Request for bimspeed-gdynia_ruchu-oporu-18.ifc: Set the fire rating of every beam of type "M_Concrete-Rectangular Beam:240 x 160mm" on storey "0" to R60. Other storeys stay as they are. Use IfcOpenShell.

First a look at what the model holds.

```python
import ifcopenshell
import ifcopenshell.util.element

model = ifcopenshell.open("bimspeed-gdynia_ruchu-oporu-18.ifc")
print(model.schema)
storey = next(s for s in model.by_type("IfcBuildingStorey") if s.Name == "0")
beams = [e for e in ifcopenshell.util.element.get_decomposition(storey) if e.is_a("IfcBeam")]
seen = {}
for e in beams:
    element_type = ifcopenshell.util.element.get_type(e)
    key = (element_type.Name if element_type != e and element_type else None, ifcopenshell.util.element.get_pset(e, "Pset_BeamCommon", "FireRating"))
    seen[key] = seen.get(key, 0) + 1
for (name, value), count in sorted(seen.items(), key=str):
    print(count, "x", name, "|", value)
```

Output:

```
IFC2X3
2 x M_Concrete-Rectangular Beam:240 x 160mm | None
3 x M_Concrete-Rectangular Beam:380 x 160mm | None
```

```python
import ifcopenshell
import ifcopenshell.api.pset
import ifcopenshell.util.element

model = ifcopenshell.open("bimspeed-gdynia_ruchu-oporu-18.ifc")

storey = next(s for s in model.by_type("IfcBuildingStorey") if s.Name == "0")
beams = [e for e in ifcopenshell.util.element.get_decomposition(storey) if e.is_a("IfcBeam")]

count = 0
for e in beams:
    element_type = ifcopenshell.util.element.get_type(e)
    if element_type in (None, e) or element_type.Name != "M_Concrete-Rectangular Beam:240 x 160mm":
        continue
    # add_pset returns the element's existing set when there is one.
    pset = ifcopenshell.api.pset.add_pset(model, product=e, name="Pset_BeamCommon")
    ifcopenshell.api.pset.edit_pset(model, pset=pset, properties={"FireRating": "R60"})
    count += 1

print(count, "beams updated")

model.write("bimspeed-gdynia_ruchu-oporu-18_updated.ifc")
```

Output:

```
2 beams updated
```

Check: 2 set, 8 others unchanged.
